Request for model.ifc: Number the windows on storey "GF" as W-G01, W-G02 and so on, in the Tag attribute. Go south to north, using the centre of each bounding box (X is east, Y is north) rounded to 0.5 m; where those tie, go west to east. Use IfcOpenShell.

First a look at what the model holds.

```python
import ifcopenshell
import ifcopenshell.util.element
import ifcopenshell.util.placement

model = ifcopenshell.open("model.ifc")
print(model.schema)
storey = next(s for s in model.by_type("IfcBuildingStorey") if s.Name == "GF")
windows = [e for e in ifcopenshell.util.element.get_decomposition(storey) if e.is_a("IfcWindow")]
for e in sorted(windows, key=lambda e: e.id()):
    origin = ifcopenshell.util.placement.get_local_placement(e.ObjectPlacement)[:3, 3]
    print(e.id(), e.Tag, e.Name, origin.round(2) + 0.0, sep=" | ")
```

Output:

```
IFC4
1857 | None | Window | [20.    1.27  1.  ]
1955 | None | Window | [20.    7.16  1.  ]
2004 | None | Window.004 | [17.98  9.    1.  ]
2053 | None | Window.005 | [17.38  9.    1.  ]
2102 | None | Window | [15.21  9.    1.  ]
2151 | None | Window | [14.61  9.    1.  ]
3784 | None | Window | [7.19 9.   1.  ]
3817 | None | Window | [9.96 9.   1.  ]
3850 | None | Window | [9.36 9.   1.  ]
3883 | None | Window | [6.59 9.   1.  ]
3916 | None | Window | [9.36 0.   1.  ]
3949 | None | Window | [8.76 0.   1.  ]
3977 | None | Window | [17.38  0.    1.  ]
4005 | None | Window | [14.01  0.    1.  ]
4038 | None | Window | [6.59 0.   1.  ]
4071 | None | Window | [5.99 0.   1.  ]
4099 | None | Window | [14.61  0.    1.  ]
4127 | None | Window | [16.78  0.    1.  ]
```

```python
import ifcopenshell
import ifcopenshell.geom
import ifcopenshell.util.element
import ifcopenshell.util.shape

model = ifcopenshell.open("model.ifc")
settings = ifcopenshell.geom.settings()
settings.set("use-world-coords", True)


def centre(element):
    shape = ifcopenshell.geom.create_shape(settings, element)
    return ifcopenshell.util.shape.get_bbox_centroid(shape.geometry)


storey = next(s for s in model.by_type("IfcBuildingStorey") if s.Name == "GF")
windows = [e for e in ifcopenshell.util.element.get_decomposition(storey) if e.is_a("IfcWindow")]

# Insertion points can sit at a corner or the storey origin, so sort by the geometry (in metres).
centres = {e: centre(e) for e in windows}
windows.sort(key=lambda e: (round(centres[e][1] / 0.5), centres[e][0]))

for i, e in enumerate(windows, start=1):
    number = f"W-G{i:02d}"
    e.Tag = number
    print(e.id(), number)

model.write("model_updated.ifc")
```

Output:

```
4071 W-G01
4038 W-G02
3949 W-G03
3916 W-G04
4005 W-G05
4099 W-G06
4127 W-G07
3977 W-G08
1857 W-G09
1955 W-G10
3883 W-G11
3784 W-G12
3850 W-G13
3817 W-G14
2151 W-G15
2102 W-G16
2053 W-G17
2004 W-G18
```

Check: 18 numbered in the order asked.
